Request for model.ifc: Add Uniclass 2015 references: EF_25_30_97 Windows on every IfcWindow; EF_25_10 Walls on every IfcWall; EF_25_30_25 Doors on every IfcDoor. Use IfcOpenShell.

First a look at what the model holds.

```python
import ifcopenshell

model = ifcopenshell.open("model.ifc")
print(model.schema)
print("classifications:", [c.Name for c in model.by_type("IfcClassification")])
for ifc_class in ("IfcDoor", "IfcRoof", "IfcStair", "IfcWall", "IfcWindow"):
    print(ifc_class, len(model.by_type(ifc_class)))
```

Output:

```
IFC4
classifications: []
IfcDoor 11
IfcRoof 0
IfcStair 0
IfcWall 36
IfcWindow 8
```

```python
import ifcopenshell
import ifcopenshell.api.classification

model = ifcopenshell.open("model.ifc")

system = ifcopenshell.api.classification.add_classification(model, classification="Uniclass 2015")

codes = {
    "IfcWindow": ("EF_25_30_97", "Windows"),
    "IfcWall": ("EF_25_10", "Walls"),
    "IfcDoor": ("EF_25_30_25", "Doors"),
}
for ifc_class, (code, name) in codes.items():
    products = model.by_type(ifc_class)
    ifcopenshell.api.classification.add_reference(
        model, products=products, classification=system, identification=code, name=name
    )
    print(code, len(products))

model.write("model-out.ifc")
```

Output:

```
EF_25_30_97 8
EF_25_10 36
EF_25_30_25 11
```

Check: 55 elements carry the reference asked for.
